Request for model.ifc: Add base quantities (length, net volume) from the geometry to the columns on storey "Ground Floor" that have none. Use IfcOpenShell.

First a look at what the model holds.

```python
import ifcopenshell
import ifcopenshell.util.element
import ifcopenshell.util.unit

model = ifcopenshell.open("model.ifc")
print(model.schema)
for unit_type in ("LENGTHUNIT", "AREAUNIT", "VOLUMEUNIT"):
    print(unit_type, ifcopenshell.util.unit.calculate_unit_scale(model, unit_type))
storey = next(s for s in model.by_type("IfcBuildingStorey") if s.Name == "Ground Floor")
columns = [e for e in ifcopenshell.util.element.get_decomposition(storey) if e.is_a("IfcColumn")]
for e in sorted(columns, key=lambda e: e.id()):
    print(e.id(), e.is_a(), e.Name, list(ifcopenshell.util.element.get_psets(e, qtos_only=True)), sep=" | ")
```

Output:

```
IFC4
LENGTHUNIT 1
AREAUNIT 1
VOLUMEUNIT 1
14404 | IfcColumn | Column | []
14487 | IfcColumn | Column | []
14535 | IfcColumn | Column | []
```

```python
import ifcopenshell
import ifcopenshell.api.pset
import ifcopenshell.geom
import ifcopenshell.util.element
import ifcopenshell.util.shape
import ifcopenshell.util.unit

model = ifcopenshell.open("model.ifc")
unit_scale = ifcopenshell.util.unit.calculate_unit_scale(model)
volume_scale = ifcopenshell.util.unit.calculate_unit_scale(model, "VOLUMEUNIT")
settings = ifcopenshell.geom.settings()

storey = next(s for s in model.by_type("IfcBuildingStorey") if s.Name == "Ground Floor")
columns = [e for e in ifcopenshell.util.element.get_decomposition(storey) if e.is_a("IfcColumn")]

for e in sorted(columns, key=lambda e: e.id()):
    if ifcopenshell.util.element.get_psets(e, qtos_only=True, should_inherit=False):
        continue
    # Geometry comes back in metres, in the element's own axes.
    shape = ifcopenshell.geom.create_shape(settings, e)
    values = {
        "Length": ifcopenshell.util.shape.get_z(shape.geometry) / unit_scale,
        "NetVolume": ifcopenshell.util.shape.get_volume(shape.geometry) / volume_scale,
    }
    qto = ifcopenshell.api.pset.add_qto(model, product=e, name="Qto_ColumnBaseQuantities")
    ifcopenshell.api.pset.edit_qto(model, qto=qto, properties=values)
    print(e.id(), {k: round(v, 3) for k, v in values.items()})

model.write("model_updated.ifc")
```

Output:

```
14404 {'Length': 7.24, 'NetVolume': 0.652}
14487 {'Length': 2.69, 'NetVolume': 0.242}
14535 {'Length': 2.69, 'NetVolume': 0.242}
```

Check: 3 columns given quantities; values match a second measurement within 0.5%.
